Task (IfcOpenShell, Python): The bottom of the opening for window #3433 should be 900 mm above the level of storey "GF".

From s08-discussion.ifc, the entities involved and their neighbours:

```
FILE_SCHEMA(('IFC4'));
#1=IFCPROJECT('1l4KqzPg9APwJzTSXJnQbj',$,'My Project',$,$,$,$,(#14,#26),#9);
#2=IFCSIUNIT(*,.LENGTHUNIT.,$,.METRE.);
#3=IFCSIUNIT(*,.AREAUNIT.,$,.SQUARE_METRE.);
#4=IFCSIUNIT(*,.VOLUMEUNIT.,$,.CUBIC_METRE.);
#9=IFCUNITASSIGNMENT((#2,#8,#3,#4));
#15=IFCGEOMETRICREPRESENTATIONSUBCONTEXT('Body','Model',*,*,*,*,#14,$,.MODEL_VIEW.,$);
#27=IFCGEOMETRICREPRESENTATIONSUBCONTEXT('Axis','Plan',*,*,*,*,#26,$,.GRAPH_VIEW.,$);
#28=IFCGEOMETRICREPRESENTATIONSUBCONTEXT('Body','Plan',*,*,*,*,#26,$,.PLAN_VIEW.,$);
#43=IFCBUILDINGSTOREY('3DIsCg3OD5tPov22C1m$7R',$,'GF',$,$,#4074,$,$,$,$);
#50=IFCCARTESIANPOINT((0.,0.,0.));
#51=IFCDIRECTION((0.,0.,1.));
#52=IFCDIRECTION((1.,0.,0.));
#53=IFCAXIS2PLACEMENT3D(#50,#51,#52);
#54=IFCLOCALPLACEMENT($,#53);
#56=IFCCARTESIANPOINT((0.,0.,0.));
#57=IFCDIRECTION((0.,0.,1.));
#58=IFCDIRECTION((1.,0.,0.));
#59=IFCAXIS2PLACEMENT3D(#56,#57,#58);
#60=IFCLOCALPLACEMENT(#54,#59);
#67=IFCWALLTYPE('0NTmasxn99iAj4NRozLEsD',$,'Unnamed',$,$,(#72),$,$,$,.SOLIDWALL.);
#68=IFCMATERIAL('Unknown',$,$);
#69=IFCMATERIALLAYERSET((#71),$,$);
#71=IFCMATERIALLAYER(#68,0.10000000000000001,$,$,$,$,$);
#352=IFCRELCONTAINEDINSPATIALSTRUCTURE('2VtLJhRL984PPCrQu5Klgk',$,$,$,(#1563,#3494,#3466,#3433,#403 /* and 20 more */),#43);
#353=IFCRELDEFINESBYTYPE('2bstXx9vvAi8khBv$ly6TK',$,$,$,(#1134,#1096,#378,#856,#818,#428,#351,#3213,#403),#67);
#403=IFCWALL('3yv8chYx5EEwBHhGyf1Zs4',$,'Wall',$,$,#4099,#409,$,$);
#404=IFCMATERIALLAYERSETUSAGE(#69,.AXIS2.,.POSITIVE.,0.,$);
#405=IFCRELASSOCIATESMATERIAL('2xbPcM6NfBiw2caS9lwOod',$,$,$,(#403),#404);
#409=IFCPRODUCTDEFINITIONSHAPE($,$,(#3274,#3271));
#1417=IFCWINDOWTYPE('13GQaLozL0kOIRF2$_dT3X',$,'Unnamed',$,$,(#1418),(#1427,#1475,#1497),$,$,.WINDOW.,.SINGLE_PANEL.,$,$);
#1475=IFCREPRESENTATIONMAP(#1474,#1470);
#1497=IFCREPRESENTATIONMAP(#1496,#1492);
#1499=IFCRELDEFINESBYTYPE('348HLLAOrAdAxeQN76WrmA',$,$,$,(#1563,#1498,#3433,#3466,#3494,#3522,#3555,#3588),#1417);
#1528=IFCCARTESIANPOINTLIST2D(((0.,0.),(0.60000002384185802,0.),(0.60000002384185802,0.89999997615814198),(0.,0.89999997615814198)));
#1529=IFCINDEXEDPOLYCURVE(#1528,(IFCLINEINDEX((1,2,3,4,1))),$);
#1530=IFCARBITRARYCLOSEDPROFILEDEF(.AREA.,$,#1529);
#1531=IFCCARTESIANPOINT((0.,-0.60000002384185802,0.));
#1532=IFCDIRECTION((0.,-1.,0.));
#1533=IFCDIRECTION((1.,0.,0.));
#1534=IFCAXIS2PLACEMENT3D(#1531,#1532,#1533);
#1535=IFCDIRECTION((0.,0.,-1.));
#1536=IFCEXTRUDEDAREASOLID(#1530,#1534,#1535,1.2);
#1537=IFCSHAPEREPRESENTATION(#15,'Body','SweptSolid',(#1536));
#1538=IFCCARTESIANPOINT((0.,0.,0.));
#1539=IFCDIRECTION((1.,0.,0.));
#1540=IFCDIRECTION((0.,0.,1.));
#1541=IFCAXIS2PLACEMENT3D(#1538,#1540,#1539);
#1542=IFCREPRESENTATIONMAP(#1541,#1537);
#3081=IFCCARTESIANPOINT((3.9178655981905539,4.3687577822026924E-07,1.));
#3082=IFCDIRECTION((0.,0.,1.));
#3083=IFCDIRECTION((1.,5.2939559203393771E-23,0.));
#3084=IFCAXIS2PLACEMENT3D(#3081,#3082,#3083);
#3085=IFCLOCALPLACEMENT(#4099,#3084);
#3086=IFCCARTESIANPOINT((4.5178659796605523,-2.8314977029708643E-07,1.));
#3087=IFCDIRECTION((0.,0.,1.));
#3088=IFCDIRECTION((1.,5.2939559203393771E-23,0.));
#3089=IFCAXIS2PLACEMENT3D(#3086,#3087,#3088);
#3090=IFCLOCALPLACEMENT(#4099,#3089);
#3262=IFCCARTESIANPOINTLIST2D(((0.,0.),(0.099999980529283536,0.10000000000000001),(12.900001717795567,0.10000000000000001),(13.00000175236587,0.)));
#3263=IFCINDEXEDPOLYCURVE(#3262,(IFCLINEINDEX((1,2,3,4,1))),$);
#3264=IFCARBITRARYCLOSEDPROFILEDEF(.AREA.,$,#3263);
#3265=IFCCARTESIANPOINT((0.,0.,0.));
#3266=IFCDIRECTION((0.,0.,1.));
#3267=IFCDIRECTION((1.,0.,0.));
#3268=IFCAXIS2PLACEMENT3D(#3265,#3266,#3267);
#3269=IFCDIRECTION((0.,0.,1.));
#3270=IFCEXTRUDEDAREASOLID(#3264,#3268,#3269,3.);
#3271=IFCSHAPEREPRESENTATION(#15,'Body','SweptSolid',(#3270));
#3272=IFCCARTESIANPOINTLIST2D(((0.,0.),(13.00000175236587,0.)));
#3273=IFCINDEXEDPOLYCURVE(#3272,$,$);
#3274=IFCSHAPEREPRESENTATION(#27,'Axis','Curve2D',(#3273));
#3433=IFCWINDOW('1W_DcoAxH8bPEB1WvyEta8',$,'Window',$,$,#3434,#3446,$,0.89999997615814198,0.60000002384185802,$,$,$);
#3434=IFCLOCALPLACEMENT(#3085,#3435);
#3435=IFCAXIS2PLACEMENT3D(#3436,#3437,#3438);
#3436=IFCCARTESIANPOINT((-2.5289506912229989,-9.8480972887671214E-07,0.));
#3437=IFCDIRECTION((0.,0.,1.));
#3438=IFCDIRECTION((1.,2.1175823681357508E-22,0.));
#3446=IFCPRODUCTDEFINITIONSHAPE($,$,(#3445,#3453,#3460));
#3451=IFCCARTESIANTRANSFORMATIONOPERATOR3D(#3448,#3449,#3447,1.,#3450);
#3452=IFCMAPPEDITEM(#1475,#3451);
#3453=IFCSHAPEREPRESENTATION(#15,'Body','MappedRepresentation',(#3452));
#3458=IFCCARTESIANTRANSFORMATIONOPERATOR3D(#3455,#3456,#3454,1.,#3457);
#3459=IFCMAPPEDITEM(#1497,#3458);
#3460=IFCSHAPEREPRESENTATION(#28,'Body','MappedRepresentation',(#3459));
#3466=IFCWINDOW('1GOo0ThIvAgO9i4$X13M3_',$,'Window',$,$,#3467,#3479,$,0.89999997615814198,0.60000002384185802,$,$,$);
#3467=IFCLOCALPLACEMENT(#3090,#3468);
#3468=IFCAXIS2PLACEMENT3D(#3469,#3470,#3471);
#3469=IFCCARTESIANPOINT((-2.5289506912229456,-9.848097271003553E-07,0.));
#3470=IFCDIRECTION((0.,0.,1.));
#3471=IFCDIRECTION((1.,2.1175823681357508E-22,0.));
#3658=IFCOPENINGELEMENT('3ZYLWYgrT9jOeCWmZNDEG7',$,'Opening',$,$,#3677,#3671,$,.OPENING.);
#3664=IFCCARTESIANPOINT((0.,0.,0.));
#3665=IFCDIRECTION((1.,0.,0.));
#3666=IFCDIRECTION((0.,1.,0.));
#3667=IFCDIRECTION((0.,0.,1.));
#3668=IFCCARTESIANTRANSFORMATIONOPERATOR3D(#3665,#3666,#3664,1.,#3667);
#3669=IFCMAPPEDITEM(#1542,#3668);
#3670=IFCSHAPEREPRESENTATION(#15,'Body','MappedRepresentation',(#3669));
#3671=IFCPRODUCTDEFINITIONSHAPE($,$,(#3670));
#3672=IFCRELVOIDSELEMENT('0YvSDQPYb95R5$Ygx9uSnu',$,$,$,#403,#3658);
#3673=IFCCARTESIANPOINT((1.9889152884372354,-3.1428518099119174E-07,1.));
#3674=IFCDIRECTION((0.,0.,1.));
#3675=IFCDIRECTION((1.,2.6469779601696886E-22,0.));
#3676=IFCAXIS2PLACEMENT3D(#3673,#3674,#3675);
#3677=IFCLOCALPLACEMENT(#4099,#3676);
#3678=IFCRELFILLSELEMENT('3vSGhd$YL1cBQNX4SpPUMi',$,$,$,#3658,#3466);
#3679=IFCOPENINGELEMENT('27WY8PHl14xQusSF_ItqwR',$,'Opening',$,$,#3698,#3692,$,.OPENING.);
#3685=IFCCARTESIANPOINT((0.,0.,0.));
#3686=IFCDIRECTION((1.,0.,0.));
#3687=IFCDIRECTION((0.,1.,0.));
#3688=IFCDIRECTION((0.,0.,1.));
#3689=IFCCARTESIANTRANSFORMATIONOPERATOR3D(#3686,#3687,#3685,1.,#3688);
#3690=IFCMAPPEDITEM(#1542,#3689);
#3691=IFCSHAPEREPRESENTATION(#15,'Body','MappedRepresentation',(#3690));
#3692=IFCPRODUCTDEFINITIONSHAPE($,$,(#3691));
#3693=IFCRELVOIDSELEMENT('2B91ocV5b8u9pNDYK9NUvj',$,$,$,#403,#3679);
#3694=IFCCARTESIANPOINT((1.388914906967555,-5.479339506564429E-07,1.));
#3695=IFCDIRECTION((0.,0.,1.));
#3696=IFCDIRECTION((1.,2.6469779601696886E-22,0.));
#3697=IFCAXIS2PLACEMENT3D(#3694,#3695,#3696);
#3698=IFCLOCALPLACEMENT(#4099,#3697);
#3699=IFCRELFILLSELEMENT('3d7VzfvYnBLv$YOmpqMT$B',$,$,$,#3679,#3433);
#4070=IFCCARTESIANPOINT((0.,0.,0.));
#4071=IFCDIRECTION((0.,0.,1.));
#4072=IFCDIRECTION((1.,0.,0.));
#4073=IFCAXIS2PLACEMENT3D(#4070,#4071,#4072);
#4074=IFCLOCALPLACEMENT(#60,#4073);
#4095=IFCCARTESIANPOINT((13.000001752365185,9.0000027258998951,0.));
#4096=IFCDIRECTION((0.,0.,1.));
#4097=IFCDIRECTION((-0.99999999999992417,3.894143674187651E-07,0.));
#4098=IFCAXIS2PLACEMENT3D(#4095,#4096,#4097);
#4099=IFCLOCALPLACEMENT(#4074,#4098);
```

```python
import numpy as np
import ifcopenshell
import ifcopenshell.api.geometry
import ifcopenshell.geom
import ifcopenshell.util.element
import ifcopenshell.util.placement
import ifcopenshell.util.shape
import ifcopenshell.util.unit

model = ifcopenshell.open("s08-discussion.ifc")
unit_scale = ifcopenshell.util.unit.calculate_unit_scale(model)

window = model.by_guid("1W_DcoAxH8bPEB1WvyEta8")
opening = window.FillsVoids[0].RelatingOpeningElement
storey = ifcopenshell.util.element.get_container(window, ifc_class="IfcBuildingStorey")
level = ifcopenshell.util.placement.get_local_placement(storey.ObjectPlacement)[2, 3]

# The opening's origin need not be at the sill, so measure its lowest point.
shape = ifcopenshell.geom.create_shape(ifcopenshell.geom.settings(), opening)
bottom = ifcopenshell.util.shape.get_shape_bottom_elevation(shape, shape.geometry) / unit_scale
dz = level + 0.9 - bottom

shift = np.array([0.0, 0.0, dz])
# The window is not placed relative to its opening, so move both.
for product in (opening, window):
    matrix = ifcopenshell.util.placement.get_local_placement(product.ObjectPlacement)
    matrix[:3, 3] += shift
    ifcopenshell.api.geometry.edit_object_placement(model, product=product, matrix=matrix, is_si=False)

print(f"moved by {dz * unit_scale:+.3f} m")

model.write("s08-discussion_rev.ifc")
```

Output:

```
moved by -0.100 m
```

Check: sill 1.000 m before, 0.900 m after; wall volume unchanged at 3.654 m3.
